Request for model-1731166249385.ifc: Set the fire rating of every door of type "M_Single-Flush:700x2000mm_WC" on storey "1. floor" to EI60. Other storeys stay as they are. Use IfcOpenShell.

First a look at what the model holds.

```python
import ifcopenshell
import ifcopenshell.util.element

model = ifcopenshell.open("model-1731166249385.ifc")
print(model.schema)
storey = next(s for s in model.by_type("IfcBuildingStorey") if s.Name == "1. floor")
doors = [e for e in ifcopenshell.util.element.get_decomposition(storey) if e.is_a("IfcDoor")]
seen = {}
for e in doors:
    element_type = ifcopenshell.util.element.get_type(e)
    key = (element_type.Name if element_type != e and element_type else None, ifcopenshell.util.element.get_pset(e, "Pset_DoorCommon", "FireRating"))
    seen[key] = seen.get(key, 0) + 1
for (name, value), count in sorted(seen.items(), key=str):
    print(count, "x", name, "|", value)
```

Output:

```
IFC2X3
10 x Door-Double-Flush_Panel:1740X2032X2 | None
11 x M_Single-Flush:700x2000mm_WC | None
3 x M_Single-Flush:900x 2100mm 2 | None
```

```python
import ifcopenshell
import ifcopenshell.api.pset
import ifcopenshell.util.element

model = ifcopenshell.open("model-1731166249385.ifc")

storey = next(s for s in model.by_type("IfcBuildingStorey") if s.Name == "1. floor")
doors = [e for e in ifcopenshell.util.element.get_decomposition(storey) if e.is_a("IfcDoor")]

count = 0
for e in doors:
    element_type = ifcopenshell.util.element.get_type(e)
    if element_type in (None, e) or element_type.Name != "M_Single-Flush:700x2000mm_WC":
        continue
    # add_pset returns the element's existing set when there is one.
    pset = ifcopenshell.api.pset.add_pset(model, product=e, name="Pset_DoorCommon")
    ifcopenshell.api.pset.edit_pset(model, pset=pset, properties={"FireRating": "EI60"})
    count += 1

print(count, "doors updated")

model.write("model-1731166249385_updated.ifc")
```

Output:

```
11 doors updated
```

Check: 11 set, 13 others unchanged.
